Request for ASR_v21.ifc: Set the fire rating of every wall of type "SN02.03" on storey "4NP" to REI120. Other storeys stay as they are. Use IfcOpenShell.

First a look at what the model holds.

```python
import ifcopenshell
import ifcopenshell.util.element

model = ifcopenshell.open("ASR_v21.ifc")
print(model.schema)
storey = next(s for s in model.by_type("IfcBuildingStorey") if s.Name == "4NP")
walls = [e for e in ifcopenshell.util.element.get_decomposition(storey) if e.is_a("IfcWall")]
seen = {}
for e in walls:
    element_type = ifcopenshell.util.element.get_type(e)
    key = (element_type.Name if element_type != e and element_type else None, ifcopenshell.util.element.get_pset(e, "Pset_WallCommon", "FireRating"))
    seen[key] = seen.get(key, 0) + 1
for (name, value), count in sorted(seen.items(), key=str):
    print(count, "x", name, "|", value)
```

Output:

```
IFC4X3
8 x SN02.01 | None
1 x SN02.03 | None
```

```python
import ifcopenshell
import ifcopenshell.api.pset
import ifcopenshell.util.element

model = ifcopenshell.open("ASR_v21.ifc")

storey = next(s for s in model.by_type("IfcBuildingStorey") if s.Name == "4NP")
walls = [e for e in ifcopenshell.util.element.get_decomposition(storey) if e.is_a("IfcWall")]

count = 0
for e in walls:
    element_type = ifcopenshell.util.element.get_type(e)
    if element_type in (None, e) or element_type.Name != "SN02.03":
        continue
    # add_pset returns the element's existing set when there is one.
    pset = ifcopenshell.api.pset.add_pset(model, product=e, name="Pset_WallCommon")
    ifcopenshell.api.pset.edit_pset(model, pset=pset, properties={"FireRating": "REI120"})
    count += 1

print(count, "walls updated")

model.write("ASR_v21-out.ifc")
```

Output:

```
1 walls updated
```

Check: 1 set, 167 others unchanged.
